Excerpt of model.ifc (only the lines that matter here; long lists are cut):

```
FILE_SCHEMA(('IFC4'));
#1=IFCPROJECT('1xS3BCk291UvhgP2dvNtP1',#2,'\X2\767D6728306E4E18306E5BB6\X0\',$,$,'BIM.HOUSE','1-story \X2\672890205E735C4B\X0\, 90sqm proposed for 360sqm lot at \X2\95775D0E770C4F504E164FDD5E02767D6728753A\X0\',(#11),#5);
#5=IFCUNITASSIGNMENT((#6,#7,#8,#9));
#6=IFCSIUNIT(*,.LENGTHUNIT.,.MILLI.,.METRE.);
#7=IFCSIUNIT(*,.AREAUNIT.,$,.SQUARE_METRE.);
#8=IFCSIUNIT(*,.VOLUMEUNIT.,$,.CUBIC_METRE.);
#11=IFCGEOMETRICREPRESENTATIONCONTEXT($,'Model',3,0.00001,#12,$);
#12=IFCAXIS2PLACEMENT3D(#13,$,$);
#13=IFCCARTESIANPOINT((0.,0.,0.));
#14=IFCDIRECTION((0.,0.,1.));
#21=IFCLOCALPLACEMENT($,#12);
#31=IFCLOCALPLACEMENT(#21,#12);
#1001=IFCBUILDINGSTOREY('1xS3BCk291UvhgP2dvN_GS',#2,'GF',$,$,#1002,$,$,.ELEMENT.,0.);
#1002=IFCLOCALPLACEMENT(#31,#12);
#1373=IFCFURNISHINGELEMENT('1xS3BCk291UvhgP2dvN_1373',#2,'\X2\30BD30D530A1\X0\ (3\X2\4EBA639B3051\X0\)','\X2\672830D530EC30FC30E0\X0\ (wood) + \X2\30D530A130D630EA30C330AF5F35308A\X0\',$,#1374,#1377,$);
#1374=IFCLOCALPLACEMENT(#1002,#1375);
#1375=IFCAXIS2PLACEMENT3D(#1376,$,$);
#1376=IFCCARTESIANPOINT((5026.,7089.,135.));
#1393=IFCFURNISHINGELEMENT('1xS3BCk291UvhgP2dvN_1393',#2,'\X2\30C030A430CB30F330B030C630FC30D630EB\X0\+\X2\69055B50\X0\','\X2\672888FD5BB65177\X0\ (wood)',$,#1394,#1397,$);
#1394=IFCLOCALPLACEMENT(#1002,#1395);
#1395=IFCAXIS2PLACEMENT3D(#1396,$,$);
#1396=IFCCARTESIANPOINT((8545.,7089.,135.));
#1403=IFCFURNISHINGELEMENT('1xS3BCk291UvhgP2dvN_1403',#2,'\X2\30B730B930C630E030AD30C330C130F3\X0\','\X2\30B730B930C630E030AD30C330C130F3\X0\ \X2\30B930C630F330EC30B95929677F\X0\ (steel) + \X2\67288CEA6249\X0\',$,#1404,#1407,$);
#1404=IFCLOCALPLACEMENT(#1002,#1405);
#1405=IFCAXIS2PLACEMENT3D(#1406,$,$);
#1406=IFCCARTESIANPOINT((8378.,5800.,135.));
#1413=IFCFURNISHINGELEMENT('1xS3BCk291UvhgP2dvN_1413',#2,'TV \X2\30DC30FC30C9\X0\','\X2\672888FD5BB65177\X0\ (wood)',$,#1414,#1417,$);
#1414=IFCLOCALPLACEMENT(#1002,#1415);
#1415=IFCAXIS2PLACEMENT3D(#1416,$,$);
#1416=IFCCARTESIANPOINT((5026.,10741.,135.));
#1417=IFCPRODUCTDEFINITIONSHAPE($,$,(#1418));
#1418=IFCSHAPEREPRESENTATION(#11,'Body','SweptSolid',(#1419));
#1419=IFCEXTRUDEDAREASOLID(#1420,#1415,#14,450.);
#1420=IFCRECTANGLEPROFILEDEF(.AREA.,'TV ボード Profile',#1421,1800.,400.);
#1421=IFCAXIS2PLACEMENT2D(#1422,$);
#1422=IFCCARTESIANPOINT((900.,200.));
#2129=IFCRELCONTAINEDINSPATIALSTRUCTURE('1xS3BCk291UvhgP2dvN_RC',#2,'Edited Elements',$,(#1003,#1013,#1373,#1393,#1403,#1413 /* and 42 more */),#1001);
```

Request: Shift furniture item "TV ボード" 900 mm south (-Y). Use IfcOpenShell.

```python
import ifcopenshell
import ifcopenshell.api.geometry
import ifcopenshell.util.placement
import ifcopenshell.util.unit

model = ifcopenshell.open("model.ifc")
unit_scale = ifcopenshell.util.unit.calculate_unit_scale(model)

item = model.by_id(1413)
matrix = ifcopenshell.util.placement.get_local_placement(item.ObjectPlacement)
matrix[1, 3] -= 0.9 / unit_scale
ifcopenshell.api.geometry.edit_object_placement(model, product=item, matrix=matrix, is_si=False)

print(ifcopenshell.util.placement.get_local_placement(item.ObjectPlacement).round(3) + 0.0)

model.write("model_updated.ifc")
```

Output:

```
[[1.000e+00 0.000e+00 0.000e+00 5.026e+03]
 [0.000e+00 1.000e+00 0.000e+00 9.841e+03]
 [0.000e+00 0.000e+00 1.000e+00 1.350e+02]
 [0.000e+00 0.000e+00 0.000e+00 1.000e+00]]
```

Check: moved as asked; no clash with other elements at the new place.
